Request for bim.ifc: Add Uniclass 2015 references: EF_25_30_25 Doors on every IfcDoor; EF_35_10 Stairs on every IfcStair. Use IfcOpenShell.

First a look at what the model holds.

```python
import ifcopenshell

model = ifcopenshell.open("bim.ifc")
print(model.schema)
print("classifications:", [c.Name for c in model.by_type("IfcClassification")])
for ifc_class in ("IfcDoor", "IfcRoof", "IfcStair", "IfcWall", "IfcWindow"):
    print(ifc_class, len(model.by_type(ifc_class)))
```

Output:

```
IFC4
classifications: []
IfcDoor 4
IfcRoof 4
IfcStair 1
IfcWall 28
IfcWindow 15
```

```python
import ifcopenshell
import ifcopenshell.api.classification

model = ifcopenshell.open("bim.ifc")

system = ifcopenshell.api.classification.add_classification(model, classification="Uniclass 2015")

codes = {
    "IfcDoor": ("EF_25_30_25", "Doors"),
    "IfcStair": ("EF_35_10", "Stairs"),
}
for ifc_class, (code, name) in codes.items():
    products = model.by_type(ifc_class)
    ifcopenshell.api.classification.add_reference(
        model, products=products, classification=system, identification=code, name=name
    )
    print(code, len(products))

model.write("bim_v2.ifc")
```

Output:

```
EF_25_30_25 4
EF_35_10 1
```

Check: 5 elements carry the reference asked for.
